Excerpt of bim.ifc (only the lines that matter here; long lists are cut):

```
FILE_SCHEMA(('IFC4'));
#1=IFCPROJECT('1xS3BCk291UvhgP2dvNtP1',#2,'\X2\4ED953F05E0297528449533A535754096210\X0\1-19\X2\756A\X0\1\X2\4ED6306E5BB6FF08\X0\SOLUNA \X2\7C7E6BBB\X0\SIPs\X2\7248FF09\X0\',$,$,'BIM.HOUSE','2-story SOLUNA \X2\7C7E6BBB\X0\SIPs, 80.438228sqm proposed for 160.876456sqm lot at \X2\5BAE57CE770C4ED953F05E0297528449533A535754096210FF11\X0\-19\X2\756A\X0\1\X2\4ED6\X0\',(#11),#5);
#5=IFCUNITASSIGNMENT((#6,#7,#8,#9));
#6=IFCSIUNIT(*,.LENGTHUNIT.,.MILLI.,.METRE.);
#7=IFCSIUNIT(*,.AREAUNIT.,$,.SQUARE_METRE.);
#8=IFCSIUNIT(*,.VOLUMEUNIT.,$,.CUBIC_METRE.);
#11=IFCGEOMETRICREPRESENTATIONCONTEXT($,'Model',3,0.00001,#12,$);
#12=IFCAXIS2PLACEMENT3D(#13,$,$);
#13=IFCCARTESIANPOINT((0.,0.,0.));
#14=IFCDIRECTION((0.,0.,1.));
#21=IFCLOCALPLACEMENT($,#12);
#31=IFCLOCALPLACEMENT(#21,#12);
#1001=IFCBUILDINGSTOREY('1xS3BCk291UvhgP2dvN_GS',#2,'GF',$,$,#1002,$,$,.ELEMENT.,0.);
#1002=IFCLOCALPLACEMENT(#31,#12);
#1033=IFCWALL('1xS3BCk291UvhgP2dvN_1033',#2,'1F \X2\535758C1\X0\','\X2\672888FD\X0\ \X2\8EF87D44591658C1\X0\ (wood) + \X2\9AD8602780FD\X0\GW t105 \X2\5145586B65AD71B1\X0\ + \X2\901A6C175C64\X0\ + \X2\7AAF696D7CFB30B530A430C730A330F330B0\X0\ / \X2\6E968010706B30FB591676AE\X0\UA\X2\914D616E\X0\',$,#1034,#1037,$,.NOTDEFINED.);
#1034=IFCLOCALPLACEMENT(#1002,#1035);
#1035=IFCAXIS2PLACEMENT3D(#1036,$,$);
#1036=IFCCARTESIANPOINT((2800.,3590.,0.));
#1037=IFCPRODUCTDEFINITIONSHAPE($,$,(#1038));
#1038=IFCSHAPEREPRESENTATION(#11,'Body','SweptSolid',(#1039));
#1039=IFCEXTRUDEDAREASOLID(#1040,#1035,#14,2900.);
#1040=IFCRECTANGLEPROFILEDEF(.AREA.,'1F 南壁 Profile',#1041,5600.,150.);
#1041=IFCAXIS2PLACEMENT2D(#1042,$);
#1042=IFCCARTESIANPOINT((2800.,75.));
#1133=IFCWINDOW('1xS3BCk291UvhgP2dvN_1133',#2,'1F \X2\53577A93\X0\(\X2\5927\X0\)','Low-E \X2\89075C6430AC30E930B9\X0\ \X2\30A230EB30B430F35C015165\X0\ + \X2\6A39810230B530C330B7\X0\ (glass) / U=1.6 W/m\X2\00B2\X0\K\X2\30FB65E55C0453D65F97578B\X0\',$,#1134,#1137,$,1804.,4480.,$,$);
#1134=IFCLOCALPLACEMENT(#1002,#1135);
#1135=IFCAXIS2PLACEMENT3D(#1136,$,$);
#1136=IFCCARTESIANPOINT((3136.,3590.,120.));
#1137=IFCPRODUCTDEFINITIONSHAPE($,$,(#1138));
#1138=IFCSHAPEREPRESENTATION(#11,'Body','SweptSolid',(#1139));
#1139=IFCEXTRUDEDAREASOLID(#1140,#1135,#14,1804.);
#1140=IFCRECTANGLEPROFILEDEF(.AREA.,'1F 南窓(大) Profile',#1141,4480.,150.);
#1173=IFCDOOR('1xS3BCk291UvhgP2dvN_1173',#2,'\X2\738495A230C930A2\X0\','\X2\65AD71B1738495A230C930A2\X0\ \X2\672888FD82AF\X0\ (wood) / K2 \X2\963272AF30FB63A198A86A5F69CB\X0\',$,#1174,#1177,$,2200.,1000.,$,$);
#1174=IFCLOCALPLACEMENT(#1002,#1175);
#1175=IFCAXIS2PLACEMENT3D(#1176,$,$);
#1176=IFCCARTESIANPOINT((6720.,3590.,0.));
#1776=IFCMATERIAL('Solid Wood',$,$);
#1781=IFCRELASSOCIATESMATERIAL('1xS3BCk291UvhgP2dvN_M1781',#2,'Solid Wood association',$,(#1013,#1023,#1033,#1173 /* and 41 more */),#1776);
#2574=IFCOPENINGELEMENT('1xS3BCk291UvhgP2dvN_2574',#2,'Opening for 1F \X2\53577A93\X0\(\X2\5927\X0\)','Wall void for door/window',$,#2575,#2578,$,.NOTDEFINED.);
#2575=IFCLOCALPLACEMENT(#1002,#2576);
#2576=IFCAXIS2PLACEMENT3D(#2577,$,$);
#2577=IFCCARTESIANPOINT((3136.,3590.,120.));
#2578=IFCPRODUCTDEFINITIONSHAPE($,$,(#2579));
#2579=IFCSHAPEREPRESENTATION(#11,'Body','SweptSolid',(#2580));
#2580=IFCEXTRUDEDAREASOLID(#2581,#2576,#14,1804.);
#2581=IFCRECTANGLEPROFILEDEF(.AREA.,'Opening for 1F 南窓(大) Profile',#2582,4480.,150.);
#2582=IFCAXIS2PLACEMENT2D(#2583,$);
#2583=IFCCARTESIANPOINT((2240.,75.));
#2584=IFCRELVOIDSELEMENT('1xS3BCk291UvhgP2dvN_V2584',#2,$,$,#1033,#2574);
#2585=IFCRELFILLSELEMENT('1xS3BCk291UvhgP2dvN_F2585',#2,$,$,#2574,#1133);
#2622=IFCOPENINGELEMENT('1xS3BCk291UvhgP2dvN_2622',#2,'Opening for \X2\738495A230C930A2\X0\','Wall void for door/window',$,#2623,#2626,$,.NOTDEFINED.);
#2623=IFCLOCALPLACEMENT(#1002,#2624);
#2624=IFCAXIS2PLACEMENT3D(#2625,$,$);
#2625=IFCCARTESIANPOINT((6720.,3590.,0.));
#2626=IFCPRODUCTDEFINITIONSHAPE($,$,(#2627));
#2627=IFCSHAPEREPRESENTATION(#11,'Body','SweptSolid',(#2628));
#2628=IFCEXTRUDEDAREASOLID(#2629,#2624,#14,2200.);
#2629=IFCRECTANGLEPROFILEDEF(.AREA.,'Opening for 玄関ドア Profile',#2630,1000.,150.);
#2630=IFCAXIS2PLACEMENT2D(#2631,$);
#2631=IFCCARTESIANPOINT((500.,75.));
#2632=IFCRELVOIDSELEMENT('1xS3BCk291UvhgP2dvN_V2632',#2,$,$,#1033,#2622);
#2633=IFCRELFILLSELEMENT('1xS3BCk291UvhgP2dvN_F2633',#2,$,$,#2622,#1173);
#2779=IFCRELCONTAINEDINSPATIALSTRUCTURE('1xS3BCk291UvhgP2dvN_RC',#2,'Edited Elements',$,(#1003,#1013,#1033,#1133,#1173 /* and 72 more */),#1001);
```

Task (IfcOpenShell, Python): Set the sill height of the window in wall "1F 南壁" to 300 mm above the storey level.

```python
import numpy as np
import ifcopenshell
import ifcopenshell.api.geometry
import ifcopenshell.geom
import ifcopenshell.util.element
import ifcopenshell.util.placement
import ifcopenshell.util.shape
import ifcopenshell.util.unit

model = ifcopenshell.open("bim.ifc")
unit_scale = ifcopenshell.util.unit.calculate_unit_scale(model)

window = model.by_id(1133)
opening = window.FillsVoids[0].RelatingOpeningElement
storey = ifcopenshell.util.element.get_container(window, ifc_class="IfcBuildingStorey")
level = ifcopenshell.util.placement.get_local_placement(storey.ObjectPlacement)[2, 3]

# The opening's origin need not be at the sill, so measure its lowest point.
shape = ifcopenshell.geom.create_shape(ifcopenshell.geom.settings(), opening)
bottom = ifcopenshell.util.shape.get_shape_bottom_elevation(shape, shape.geometry) / unit_scale
dz = level + 300.0 - bottom

shift = np.array([0.0, 0.0, dz])
# The window is not placed relative to its opening, so move both.
for product in (opening, window):
    matrix = ifcopenshell.util.placement.get_local_placement(product.ObjectPlacement)
    matrix[:3, 3] += shift
    ifcopenshell.api.geometry.edit_object_placement(model, product=product, matrix=matrix, is_si=False)

print(f"moved by {dz * unit_scale:+.3f} m")

model.write("bim_updated.ifc")
```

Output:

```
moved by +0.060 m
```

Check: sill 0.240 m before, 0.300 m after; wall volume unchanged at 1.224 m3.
